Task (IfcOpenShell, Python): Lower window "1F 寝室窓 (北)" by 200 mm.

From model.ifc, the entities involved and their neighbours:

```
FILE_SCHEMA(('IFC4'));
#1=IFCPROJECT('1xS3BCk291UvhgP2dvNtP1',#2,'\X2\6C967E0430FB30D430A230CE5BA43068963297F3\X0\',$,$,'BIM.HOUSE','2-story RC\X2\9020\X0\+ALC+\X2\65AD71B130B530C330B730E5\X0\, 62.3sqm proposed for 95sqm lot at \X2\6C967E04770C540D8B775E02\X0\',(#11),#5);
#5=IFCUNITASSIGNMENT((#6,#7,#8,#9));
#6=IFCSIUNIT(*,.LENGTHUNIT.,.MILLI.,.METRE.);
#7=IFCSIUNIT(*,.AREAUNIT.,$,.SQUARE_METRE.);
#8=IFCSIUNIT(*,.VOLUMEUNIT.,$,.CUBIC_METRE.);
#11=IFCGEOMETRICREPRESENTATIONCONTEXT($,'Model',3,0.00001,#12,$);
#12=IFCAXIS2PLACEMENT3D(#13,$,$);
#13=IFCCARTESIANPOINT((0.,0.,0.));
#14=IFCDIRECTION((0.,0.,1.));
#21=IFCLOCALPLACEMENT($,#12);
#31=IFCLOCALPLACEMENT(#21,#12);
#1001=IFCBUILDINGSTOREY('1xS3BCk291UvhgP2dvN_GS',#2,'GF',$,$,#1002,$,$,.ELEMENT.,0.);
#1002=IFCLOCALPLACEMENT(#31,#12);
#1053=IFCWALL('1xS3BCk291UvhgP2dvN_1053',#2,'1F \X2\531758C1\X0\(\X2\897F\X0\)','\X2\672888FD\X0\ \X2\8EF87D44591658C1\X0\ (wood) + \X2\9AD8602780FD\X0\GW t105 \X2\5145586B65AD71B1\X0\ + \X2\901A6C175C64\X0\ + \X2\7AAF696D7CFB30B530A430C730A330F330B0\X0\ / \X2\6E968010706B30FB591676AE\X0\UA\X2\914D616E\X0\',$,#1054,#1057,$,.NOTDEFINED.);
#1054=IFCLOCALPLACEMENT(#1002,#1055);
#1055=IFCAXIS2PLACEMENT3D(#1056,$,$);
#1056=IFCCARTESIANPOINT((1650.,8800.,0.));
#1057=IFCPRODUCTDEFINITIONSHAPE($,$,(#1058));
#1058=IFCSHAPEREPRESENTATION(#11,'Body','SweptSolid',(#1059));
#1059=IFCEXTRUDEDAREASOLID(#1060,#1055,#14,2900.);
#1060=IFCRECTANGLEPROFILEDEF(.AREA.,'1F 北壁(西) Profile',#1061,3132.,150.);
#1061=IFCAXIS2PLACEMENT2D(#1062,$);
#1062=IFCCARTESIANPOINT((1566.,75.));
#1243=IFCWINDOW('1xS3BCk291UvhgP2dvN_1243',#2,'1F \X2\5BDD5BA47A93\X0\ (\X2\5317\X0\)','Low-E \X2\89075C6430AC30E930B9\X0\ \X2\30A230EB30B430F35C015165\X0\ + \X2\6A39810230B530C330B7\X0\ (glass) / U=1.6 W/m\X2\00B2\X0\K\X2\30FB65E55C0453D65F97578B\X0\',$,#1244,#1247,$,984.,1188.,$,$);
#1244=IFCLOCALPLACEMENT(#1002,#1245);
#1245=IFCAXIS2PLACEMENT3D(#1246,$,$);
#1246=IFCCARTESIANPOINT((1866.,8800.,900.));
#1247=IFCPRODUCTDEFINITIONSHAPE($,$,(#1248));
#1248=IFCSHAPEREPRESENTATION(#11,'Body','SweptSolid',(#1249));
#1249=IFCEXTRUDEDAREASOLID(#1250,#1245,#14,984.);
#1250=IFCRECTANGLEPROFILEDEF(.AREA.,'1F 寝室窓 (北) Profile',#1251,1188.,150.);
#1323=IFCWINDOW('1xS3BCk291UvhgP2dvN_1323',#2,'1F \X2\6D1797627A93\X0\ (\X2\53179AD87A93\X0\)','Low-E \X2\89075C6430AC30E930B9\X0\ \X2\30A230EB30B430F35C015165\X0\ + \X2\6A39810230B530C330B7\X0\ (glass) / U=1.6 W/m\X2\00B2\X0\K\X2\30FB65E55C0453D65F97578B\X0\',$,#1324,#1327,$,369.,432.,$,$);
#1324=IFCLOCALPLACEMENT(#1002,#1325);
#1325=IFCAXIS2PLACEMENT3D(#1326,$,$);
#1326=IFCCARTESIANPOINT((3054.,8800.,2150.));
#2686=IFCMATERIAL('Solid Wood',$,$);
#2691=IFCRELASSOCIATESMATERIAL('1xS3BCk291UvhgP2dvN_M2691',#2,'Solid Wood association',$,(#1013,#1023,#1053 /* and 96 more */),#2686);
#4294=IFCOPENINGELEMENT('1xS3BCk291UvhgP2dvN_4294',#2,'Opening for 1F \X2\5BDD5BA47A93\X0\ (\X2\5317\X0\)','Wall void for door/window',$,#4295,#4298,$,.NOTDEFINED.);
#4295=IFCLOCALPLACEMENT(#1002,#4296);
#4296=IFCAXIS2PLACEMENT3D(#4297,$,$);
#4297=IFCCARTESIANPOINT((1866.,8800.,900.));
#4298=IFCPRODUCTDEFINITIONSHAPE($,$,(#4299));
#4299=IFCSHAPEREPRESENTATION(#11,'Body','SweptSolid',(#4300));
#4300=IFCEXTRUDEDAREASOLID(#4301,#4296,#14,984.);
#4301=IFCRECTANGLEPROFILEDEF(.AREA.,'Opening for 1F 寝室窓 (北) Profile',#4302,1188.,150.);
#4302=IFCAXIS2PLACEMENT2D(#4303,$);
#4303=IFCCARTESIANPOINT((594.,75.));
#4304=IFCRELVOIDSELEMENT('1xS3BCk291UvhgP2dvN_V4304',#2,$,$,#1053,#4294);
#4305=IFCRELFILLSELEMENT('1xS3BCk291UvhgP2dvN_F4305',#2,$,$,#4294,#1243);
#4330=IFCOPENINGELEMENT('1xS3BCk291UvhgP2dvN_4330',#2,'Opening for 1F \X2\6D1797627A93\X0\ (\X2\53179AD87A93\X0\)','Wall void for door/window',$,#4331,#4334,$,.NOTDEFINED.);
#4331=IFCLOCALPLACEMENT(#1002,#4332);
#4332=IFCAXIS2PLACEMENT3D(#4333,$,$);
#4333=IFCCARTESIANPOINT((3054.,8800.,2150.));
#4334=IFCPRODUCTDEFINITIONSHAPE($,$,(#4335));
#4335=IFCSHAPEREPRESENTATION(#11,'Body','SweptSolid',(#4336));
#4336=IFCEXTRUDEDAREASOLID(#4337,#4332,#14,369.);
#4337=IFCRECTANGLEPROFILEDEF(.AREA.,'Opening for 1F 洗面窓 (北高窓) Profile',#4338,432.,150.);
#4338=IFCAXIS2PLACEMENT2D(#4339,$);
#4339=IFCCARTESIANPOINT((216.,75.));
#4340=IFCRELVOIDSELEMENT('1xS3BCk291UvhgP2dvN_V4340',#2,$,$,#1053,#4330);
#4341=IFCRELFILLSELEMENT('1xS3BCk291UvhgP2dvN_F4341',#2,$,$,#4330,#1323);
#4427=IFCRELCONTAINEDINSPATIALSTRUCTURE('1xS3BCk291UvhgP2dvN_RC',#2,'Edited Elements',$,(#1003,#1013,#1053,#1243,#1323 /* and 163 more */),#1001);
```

```python
import numpy as np
import ifcopenshell
import ifcopenshell.api.geometry
import ifcopenshell.util.placement
import ifcopenshell.util.unit

model = ifcopenshell.open("model.ifc")
unit_scale = ifcopenshell.util.unit.calculate_unit_scale(model)

window = model.by_id(1243)
opening = window.FillsVoids[0].RelatingOpeningElement
dz = -0.2 / unit_scale

shift = np.array([0.0, 0.0, dz])
# The window is not placed relative to its opening, so move both.
for product in (opening, window):
    matrix = ifcopenshell.util.placement.get_local_placement(product.ObjectPlacement)
    matrix[:3, 3] += shift
    ifcopenshell.api.geometry.edit_object_placement(model, product=product, matrix=matrix, is_si=False)

print(f"moved by {dz * unit_scale:+.3f} m")

model.write("model_v2.ifc")
```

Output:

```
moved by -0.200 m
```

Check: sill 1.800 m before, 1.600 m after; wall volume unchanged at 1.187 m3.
